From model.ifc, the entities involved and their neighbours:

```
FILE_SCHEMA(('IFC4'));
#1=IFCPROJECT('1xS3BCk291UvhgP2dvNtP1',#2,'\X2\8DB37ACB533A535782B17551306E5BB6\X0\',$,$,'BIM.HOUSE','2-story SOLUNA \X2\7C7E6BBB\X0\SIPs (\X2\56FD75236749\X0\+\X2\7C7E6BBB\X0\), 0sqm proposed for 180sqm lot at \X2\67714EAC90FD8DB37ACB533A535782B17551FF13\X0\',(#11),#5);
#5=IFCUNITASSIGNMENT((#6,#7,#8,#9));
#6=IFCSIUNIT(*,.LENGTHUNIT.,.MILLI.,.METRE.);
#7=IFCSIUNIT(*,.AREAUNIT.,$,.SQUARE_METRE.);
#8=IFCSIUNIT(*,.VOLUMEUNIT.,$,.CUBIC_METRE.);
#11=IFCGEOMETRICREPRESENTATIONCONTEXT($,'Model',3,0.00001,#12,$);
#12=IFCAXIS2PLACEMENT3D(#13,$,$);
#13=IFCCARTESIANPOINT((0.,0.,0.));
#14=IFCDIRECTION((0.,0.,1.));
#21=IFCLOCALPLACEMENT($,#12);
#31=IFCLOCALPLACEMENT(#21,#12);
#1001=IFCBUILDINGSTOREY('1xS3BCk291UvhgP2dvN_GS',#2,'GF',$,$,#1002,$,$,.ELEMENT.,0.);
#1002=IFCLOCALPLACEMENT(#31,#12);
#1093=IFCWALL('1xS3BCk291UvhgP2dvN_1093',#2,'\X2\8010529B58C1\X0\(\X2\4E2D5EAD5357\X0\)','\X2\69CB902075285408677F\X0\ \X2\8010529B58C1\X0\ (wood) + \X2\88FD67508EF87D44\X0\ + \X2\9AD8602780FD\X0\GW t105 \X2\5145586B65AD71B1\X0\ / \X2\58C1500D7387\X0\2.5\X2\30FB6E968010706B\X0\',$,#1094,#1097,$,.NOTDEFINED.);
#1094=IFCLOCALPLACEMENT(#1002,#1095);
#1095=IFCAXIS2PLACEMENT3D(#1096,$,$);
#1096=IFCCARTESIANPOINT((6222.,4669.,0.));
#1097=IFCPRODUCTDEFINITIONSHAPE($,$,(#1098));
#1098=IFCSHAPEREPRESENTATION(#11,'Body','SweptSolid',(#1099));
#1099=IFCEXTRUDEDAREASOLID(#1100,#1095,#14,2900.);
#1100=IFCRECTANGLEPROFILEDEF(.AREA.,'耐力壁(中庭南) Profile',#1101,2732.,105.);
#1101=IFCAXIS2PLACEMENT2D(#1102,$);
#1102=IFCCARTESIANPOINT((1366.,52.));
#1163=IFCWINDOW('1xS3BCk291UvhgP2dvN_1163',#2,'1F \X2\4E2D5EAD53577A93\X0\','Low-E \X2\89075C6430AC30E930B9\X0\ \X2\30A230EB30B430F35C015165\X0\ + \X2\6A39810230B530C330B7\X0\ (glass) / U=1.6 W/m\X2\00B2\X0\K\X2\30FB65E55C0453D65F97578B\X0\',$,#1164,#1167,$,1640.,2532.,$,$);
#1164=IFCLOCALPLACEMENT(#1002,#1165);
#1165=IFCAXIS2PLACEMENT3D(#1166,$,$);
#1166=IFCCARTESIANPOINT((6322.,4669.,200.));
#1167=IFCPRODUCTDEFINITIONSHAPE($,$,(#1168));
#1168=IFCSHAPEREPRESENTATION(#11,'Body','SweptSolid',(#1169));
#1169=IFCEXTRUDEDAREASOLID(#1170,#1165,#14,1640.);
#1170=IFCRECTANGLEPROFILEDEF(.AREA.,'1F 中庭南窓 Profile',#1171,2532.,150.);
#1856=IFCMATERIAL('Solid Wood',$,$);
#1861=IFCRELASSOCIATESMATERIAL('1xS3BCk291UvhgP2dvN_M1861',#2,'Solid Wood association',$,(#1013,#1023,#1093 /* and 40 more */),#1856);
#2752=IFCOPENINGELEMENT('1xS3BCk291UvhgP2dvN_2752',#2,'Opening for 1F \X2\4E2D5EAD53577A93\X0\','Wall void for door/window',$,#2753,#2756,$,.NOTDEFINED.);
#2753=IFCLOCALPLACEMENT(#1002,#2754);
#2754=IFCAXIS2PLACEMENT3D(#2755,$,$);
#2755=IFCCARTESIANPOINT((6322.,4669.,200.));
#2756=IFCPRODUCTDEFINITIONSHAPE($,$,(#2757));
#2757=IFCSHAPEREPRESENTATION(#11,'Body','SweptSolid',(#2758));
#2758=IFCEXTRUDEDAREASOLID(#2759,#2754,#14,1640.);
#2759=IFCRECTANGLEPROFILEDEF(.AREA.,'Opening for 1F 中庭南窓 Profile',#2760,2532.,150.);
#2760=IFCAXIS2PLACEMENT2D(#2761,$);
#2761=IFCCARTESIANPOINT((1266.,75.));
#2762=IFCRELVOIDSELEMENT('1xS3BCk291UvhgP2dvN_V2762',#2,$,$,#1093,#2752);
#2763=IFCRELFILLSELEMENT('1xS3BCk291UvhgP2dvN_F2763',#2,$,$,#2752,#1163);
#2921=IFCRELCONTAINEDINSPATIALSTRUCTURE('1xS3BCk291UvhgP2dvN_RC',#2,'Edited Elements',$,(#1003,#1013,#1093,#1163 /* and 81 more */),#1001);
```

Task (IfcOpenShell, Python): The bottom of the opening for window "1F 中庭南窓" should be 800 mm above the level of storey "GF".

```python
import numpy as np
import ifcopenshell
import ifcopenshell.api.geometry
import ifcopenshell.geom
import ifcopenshell.util.element
import ifcopenshell.util.placement
import ifcopenshell.util.shape
import ifcopenshell.util.unit

model = ifcopenshell.open("model.ifc")
unit_scale = ifcopenshell.util.unit.calculate_unit_scale(model)

window = model.by_guid("1xS3BCk291UvhgP2dvN_1163")
opening = window.FillsVoids[0].RelatingOpeningElement
storey = ifcopenshell.util.element.get_container(window, ifc_class="IfcBuildingStorey")
level = ifcopenshell.util.placement.get_local_placement(storey.ObjectPlacement)[2, 3]

# The opening's origin need not be at the sill, so measure its lowest point.
shape = ifcopenshell.geom.create_shape(ifcopenshell.geom.settings(), opening)
bottom = ifcopenshell.util.shape.get_shape_bottom_elevation(shape, shape.geometry) / unit_scale
dz = level + 0.8 / unit_scale - bottom

shift = np.array([0.0, 0.0, dz])
# The window is not placed relative to its opening, so move both.
for product in (opening, window):
    matrix = ifcopenshell.util.placement.get_local_placement(product.ObjectPlacement)
    matrix[:3, 3] += shift
    ifcopenshell.api.geometry.edit_object_placement(model, product=product, matrix=matrix, is_si=False)

print(f"moved by {dz * unit_scale:+.3f} m")

model.write("model_v2.ifc")
```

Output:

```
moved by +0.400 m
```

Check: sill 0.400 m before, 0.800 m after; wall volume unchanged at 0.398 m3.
